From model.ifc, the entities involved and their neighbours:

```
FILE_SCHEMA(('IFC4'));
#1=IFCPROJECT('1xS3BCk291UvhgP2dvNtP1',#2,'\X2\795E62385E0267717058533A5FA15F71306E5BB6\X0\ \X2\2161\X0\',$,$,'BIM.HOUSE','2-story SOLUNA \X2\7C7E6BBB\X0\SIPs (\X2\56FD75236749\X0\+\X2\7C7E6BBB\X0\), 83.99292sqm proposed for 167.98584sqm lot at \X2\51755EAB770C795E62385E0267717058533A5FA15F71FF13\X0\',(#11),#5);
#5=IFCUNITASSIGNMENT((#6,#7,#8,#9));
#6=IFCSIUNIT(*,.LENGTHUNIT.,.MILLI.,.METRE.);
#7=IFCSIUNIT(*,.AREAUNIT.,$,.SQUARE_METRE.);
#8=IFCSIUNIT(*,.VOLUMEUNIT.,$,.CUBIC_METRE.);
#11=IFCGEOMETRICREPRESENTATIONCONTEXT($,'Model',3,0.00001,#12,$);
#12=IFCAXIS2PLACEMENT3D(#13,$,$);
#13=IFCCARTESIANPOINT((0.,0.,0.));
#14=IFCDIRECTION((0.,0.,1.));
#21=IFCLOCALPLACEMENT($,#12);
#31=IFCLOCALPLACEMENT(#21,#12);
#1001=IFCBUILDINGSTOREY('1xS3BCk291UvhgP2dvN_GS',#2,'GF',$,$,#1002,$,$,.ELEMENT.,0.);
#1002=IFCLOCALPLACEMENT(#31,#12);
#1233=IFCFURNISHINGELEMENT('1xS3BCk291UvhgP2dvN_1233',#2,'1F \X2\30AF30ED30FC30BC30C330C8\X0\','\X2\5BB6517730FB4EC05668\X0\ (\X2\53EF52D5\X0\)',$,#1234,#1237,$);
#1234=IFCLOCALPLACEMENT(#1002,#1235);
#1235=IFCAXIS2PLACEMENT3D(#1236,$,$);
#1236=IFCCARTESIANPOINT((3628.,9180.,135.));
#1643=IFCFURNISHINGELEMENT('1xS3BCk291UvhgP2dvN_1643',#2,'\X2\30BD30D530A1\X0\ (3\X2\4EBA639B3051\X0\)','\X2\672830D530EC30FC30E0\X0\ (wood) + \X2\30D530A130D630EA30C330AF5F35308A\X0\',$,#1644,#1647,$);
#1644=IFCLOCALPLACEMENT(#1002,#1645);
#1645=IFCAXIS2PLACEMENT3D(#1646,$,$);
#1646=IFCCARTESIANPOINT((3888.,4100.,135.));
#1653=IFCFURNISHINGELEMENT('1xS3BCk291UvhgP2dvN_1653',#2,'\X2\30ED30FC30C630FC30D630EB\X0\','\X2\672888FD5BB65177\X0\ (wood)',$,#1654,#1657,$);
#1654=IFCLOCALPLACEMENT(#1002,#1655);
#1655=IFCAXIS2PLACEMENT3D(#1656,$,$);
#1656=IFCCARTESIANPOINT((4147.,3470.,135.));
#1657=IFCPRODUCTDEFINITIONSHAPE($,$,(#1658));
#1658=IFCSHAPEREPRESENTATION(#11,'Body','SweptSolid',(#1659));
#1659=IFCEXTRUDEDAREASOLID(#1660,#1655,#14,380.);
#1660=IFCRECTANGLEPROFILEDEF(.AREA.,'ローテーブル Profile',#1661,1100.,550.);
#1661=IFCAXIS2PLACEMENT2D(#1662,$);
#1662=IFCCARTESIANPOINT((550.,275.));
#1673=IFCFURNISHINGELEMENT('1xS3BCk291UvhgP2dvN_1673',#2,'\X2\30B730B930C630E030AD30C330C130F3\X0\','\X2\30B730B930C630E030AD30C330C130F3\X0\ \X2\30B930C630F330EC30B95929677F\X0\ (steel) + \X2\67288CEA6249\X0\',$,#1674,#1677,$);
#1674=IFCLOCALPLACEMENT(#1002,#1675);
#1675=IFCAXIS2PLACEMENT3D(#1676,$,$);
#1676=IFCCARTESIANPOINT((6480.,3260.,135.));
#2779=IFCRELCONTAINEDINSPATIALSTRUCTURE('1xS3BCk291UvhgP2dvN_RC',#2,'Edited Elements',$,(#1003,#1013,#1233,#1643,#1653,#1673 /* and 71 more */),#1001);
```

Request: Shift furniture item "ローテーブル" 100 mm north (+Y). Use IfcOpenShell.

```python
import ifcopenshell
import ifcopenshell.api.geometry
import ifcopenshell.util.placement

model = ifcopenshell.open("model.ifc")

item = model.by_guid("1xS3BCk291UvhgP2dvN_1653")
matrix = ifcopenshell.util.placement.get_local_placement(item.ObjectPlacement)
matrix[1, 3] += 100.0
ifcopenshell.api.geometry.edit_object_placement(model, product=item, matrix=matrix, is_si=False)

print(ifcopenshell.util.placement.get_local_placement(item.ObjectPlacement).round(3) + 0.0)

model.write("model-out.ifc")
```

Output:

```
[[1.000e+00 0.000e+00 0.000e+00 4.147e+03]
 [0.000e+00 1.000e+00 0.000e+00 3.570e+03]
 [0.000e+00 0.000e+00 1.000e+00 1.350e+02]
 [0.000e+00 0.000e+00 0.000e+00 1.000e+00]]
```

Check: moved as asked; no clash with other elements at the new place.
